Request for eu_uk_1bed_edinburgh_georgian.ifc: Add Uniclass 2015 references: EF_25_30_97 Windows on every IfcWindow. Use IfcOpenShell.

First a look at what the model holds.

```python
import ifcopenshell

model = ifcopenshell.open("eu_uk_1bed_edinburgh_georgian.ifc")
print(model.schema)
print("classifications:", [c.Name for c in model.by_type("IfcClassification")])
for ifc_class in ("IfcDoor", "IfcRoof", "IfcStair", "IfcWall", "IfcWindow"):
    print(ifc_class, len(model.by_type(ifc_class)))
```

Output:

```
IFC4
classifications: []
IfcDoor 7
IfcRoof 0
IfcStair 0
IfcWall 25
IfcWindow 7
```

```python
import ifcopenshell
import ifcopenshell.api.classification

model = ifcopenshell.open("eu_uk_1bed_edinburgh_georgian.ifc")

system = ifcopenshell.api.classification.add_classification(model, classification="Uniclass 2015")

codes = {
    "IfcWindow": ("EF_25_30_97", "Windows"),
}
for ifc_class, (code, name) in codes.items():
    products = model.by_type(ifc_class)
    ifcopenshell.api.classification.add_reference(
        model, products=products, classification=system, identification=code, name=name
    )
    print(code, len(products))

model.write("eu_uk_1bed_edinburgh_georgian_updated.ifc")
```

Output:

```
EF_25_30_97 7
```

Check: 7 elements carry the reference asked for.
